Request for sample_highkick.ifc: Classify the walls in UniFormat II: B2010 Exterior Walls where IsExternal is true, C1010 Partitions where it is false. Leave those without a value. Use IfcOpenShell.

First a look at what the model holds.

```python
import ifcopenshell
import ifcopenshell.util.element

model = ifcopenshell.open("sample_highkick.ifc")
print(model.schema)
print("classifications:", [c.Name for c in model.by_type("IfcClassification")])
values = [ifcopenshell.util.element.get_pset(e, "Pset_WallCommon", "IsExternal") for e in model.by_type("IfcWall")]
for value in (True, False, None):
    print("IsExternal", value, values.count(value))
```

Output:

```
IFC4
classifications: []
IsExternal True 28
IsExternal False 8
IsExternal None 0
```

```python
import ifcopenshell
import ifcopenshell.api.classification
import ifcopenshell.util.element

model = ifcopenshell.open("sample_highkick.ifc")

system = ifcopenshell.api.classification.add_classification(model, classification="UniFormat II")

walls = model.by_type("IfcWall")
external = {e: ifcopenshell.util.element.get_pset(e, "Pset_WallCommon", "IsExternal") for e in walls}
for flag, code, name in ((True, "B2010", "Exterior Walls"), (False, "C1010", "Partitions")):
    products = [e for e in walls if external[e] is flag]
    ifcopenshell.api.classification.add_reference(
        model, products=products, classification=system, identification=code, name=name
    )
    print(code, len(products))

model.write("sample_highkick-out.ifc")
```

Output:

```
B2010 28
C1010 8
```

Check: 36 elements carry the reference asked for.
